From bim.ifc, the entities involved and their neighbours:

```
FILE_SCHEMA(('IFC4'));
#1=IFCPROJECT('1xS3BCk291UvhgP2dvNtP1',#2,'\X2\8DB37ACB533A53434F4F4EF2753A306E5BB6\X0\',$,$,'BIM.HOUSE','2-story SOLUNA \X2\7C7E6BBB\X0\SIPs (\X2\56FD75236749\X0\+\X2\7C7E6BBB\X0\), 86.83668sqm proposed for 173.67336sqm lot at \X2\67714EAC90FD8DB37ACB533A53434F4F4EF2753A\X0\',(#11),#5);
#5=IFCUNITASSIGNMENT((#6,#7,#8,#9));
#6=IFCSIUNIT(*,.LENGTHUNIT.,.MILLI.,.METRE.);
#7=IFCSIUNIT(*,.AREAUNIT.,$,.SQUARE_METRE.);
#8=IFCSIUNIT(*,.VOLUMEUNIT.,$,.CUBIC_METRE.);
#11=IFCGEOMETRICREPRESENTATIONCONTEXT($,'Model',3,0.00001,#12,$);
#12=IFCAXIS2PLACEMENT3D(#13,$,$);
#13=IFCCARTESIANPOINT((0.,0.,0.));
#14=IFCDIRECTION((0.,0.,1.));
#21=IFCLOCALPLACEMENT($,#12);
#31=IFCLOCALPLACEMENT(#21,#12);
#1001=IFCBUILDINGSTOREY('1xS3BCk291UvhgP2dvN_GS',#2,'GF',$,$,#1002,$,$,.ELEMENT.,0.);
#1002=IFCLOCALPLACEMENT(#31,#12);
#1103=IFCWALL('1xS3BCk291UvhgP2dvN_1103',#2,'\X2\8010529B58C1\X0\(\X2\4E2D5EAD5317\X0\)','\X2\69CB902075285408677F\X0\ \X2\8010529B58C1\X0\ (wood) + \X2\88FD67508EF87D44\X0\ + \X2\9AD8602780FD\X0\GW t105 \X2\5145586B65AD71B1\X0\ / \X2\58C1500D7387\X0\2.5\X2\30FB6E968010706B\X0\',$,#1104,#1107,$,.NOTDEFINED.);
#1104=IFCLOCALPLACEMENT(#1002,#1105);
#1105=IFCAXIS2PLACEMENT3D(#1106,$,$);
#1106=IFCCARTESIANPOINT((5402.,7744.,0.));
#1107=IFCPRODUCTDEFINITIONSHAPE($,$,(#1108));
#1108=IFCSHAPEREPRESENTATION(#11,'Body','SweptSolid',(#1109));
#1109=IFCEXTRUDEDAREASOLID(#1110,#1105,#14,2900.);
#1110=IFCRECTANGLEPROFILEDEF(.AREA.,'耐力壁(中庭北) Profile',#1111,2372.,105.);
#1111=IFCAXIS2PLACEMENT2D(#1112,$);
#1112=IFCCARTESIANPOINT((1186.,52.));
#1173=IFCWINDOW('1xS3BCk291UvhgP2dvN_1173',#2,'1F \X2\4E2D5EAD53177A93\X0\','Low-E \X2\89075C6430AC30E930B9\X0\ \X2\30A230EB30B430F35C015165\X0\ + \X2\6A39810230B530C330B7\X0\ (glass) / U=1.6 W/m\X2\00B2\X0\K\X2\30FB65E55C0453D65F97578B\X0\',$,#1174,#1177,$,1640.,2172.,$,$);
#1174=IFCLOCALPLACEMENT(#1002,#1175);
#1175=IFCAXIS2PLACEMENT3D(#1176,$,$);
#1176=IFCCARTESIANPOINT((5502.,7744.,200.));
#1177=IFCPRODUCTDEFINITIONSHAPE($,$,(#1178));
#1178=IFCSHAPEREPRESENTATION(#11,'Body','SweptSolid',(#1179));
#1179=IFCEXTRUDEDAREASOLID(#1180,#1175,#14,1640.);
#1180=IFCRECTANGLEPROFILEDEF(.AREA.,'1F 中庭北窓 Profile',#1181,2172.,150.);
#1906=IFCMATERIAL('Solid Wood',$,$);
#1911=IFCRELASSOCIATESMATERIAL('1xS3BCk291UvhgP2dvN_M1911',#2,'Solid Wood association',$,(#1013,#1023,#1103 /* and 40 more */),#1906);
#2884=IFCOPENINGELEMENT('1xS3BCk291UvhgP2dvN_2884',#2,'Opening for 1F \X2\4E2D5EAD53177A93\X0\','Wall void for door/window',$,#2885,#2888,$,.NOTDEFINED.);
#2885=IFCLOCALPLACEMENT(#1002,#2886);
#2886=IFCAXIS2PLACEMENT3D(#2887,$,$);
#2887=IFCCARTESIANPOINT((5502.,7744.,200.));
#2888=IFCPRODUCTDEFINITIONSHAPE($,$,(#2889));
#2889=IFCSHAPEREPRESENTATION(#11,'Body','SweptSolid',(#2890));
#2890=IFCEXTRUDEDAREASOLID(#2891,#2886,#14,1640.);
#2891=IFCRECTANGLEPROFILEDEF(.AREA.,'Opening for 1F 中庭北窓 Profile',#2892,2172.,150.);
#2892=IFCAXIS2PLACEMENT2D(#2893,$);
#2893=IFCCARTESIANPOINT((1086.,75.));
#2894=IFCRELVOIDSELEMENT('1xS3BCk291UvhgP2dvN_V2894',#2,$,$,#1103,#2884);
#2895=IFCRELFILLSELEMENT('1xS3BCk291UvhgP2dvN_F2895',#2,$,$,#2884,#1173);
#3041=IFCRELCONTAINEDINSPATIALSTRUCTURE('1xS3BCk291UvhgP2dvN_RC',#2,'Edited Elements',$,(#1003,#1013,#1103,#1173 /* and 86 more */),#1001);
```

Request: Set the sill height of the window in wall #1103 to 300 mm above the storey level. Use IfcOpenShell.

```python
import numpy as np
import ifcopenshell
import ifcopenshell.api.geometry
import ifcopenshell.geom
import ifcopenshell.util.element
import ifcopenshell.util.placement
import ifcopenshell.util.shape
import ifcopenshell.util.unit

model = ifcopenshell.open("bim.ifc")
unit_scale = ifcopenshell.util.unit.calculate_unit_scale(model)

window = model.by_guid("1xS3BCk291UvhgP2dvN_1173")
opening = window.FillsVoids[0].RelatingOpeningElement
storey = ifcopenshell.util.element.get_container(window, ifc_class="IfcBuildingStorey")
level = ifcopenshell.util.placement.get_local_placement(storey.ObjectPlacement)[2, 3]

# The opening's origin need not be at the sill, so measure its lowest point.
shape = ifcopenshell.geom.create_shape(ifcopenshell.geom.settings(), opening)
bottom = ifcopenshell.util.shape.get_shape_bottom_elevation(shape, shape.geometry) / unit_scale
dz = level + 0.3 / unit_scale - bottom

shift = np.array([0.0, 0.0, dz])
# The window is not placed relative to its opening, so move both.
for product in (opening, window):
    matrix = ifcopenshell.util.placement.get_local_placement(product.ObjectPlacement)
    matrix[:3, 3] += shift
    ifcopenshell.api.geometry.edit_object_placement(model, product=product, matrix=matrix, is_si=False)

print(f"moved by {dz * unit_scale:+.3f} m")

model.write("bim_updated.ifc")
```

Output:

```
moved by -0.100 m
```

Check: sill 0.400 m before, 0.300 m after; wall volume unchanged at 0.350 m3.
